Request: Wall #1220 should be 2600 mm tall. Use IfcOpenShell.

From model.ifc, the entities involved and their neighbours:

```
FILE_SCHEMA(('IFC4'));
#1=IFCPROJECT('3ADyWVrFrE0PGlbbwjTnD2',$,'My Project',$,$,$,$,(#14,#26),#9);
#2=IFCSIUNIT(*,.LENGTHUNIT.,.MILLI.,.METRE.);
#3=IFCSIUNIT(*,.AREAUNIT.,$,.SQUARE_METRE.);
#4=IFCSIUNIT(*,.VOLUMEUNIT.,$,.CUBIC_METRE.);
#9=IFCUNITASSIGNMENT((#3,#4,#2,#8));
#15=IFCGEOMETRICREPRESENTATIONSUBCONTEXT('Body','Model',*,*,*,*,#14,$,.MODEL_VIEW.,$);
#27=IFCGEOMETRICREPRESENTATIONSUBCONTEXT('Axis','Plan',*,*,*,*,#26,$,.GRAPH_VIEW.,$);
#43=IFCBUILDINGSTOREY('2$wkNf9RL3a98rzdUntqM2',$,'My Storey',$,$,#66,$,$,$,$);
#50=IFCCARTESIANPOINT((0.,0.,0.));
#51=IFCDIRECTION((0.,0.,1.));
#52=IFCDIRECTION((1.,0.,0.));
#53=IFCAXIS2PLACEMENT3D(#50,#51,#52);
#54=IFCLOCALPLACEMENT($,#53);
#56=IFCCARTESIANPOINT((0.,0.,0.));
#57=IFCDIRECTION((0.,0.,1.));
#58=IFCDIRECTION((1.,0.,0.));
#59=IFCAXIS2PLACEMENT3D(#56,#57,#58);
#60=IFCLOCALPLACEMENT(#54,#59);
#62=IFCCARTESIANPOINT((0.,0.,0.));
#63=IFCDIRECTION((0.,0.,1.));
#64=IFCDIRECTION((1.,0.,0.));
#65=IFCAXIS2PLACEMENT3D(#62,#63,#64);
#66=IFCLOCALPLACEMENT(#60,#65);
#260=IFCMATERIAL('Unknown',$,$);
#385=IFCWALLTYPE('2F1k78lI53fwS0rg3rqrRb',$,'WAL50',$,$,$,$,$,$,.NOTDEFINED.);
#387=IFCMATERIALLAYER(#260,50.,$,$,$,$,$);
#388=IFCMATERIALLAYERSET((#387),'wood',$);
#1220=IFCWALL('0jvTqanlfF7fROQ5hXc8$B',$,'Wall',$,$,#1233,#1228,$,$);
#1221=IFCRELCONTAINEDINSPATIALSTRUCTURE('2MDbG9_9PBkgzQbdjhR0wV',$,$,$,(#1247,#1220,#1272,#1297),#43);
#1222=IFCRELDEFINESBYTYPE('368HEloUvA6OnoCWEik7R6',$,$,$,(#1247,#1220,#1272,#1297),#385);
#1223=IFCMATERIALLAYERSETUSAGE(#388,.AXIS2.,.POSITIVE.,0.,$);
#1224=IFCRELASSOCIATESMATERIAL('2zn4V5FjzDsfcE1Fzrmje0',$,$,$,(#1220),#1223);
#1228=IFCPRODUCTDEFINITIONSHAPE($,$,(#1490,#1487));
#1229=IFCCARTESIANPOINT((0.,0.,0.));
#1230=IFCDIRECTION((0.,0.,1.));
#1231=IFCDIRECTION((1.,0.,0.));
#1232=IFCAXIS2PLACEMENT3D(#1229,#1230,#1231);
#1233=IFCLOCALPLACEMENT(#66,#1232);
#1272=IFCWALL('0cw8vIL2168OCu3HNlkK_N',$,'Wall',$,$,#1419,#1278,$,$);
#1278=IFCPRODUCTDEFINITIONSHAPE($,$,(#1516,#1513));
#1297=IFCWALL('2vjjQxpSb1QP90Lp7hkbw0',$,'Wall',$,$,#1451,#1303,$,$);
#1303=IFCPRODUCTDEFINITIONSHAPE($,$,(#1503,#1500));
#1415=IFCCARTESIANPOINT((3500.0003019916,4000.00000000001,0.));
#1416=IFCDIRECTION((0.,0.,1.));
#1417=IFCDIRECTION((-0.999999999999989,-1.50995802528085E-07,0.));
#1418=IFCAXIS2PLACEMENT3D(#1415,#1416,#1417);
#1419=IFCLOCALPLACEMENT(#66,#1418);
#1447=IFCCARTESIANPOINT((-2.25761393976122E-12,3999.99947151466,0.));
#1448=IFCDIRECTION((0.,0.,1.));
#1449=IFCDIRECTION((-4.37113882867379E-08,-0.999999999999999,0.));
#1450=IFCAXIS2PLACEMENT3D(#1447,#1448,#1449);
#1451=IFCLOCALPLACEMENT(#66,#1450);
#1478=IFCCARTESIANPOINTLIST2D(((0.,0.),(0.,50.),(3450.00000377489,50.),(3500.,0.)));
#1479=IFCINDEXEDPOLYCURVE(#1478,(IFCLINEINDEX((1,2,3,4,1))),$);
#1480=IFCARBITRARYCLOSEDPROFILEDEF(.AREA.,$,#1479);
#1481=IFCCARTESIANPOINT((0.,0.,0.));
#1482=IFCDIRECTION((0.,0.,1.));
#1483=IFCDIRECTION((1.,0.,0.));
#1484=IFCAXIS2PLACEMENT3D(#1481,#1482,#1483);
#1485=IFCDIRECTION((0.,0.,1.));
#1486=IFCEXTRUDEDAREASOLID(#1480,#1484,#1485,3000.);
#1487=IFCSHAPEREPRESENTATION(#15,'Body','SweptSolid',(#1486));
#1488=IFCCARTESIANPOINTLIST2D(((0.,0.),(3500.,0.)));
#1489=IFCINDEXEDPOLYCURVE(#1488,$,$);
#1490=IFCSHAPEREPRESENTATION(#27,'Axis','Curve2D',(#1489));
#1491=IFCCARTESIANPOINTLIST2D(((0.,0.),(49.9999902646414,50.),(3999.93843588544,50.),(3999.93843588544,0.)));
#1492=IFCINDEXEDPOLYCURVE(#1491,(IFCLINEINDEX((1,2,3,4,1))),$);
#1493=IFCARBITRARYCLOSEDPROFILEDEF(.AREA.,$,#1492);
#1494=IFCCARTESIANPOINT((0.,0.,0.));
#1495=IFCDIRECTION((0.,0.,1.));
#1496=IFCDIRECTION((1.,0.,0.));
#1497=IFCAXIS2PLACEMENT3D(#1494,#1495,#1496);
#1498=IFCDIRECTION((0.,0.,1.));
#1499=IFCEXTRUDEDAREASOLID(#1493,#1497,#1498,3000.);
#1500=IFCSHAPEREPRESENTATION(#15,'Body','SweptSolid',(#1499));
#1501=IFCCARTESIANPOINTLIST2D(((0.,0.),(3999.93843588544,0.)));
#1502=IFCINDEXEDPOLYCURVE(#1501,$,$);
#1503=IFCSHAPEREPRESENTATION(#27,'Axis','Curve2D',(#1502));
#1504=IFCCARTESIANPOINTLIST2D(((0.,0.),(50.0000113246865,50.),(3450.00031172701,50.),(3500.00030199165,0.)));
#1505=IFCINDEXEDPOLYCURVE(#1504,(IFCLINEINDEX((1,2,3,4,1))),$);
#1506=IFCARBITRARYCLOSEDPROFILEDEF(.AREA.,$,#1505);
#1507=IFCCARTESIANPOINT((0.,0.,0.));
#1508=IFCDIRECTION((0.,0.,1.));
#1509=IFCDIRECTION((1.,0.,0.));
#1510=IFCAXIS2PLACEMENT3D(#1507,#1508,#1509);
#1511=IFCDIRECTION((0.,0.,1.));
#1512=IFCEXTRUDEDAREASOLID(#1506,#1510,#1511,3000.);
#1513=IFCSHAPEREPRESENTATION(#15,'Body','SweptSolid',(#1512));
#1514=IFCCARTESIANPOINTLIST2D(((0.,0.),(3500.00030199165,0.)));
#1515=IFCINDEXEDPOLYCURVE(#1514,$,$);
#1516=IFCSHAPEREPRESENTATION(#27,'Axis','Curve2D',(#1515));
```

```python
import ifcopenshell
import ifcopenshell.geom
import ifcopenshell.util.representation
import ifcopenshell.util.shape

model = ifcopenshell.open("model.ifc")
settings = ifcopenshell.geom.settings()


def volume(element):
    """Net volume in cubic metres, openings subtracted."""
    shape = ifcopenshell.geom.create_shape(settings, element)
    return ifcopenshell.util.shape.get_volume(shape.geometry)


wall = model.by_id(1220)
before = volume(wall)

body = ifcopenshell.util.representation.get_representation(wall, "Model", "Body")
solid = body.Items[0]
old_height = solid.Depth
solid.Depth = 2600.0
after = volume(wall)

print(f"height {old_height:g} -> {solid.Depth:g}, volume {before:.3f} -> {after:.3f} m3")

model.write("model_updated.ifc")
```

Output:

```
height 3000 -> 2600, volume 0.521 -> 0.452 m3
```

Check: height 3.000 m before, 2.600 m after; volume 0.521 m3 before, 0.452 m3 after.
